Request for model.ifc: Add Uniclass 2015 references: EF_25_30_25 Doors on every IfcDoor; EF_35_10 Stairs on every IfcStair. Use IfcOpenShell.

First a look at what the model holds.

```python
import ifcopenshell

model = ifcopenshell.open("model.ifc")
print(model.schema)
print("classifications:", [c.Name for c in model.by_type("IfcClassification")])
for ifc_class in ("IfcDoor", "IfcRoof", "IfcStair", "IfcWall", "IfcWindow"):
    print(ifc_class, len(model.by_type(ifc_class)))
```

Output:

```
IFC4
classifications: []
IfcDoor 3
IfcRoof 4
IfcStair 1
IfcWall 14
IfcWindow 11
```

```python
import ifcopenshell
import ifcopenshell.api.classification

model = ifcopenshell.open("model.ifc")

system = ifcopenshell.api.classification.add_classification(model, classification="Uniclass 2015")

codes = {
    "IfcDoor": ("EF_25_30_25", "Doors"),
    "IfcStair": ("EF_35_10", "Stairs"),
}
for ifc_class, (code, name) in codes.items():
    products = model.by_type(ifc_class)
    ifcopenshell.api.classification.add_reference(
        model, products=products, classification=system, identification=code, name=name
    )
    print(code, len(products))

model.write("model_v2.ifc")
```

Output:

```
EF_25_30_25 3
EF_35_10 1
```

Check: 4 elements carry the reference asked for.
